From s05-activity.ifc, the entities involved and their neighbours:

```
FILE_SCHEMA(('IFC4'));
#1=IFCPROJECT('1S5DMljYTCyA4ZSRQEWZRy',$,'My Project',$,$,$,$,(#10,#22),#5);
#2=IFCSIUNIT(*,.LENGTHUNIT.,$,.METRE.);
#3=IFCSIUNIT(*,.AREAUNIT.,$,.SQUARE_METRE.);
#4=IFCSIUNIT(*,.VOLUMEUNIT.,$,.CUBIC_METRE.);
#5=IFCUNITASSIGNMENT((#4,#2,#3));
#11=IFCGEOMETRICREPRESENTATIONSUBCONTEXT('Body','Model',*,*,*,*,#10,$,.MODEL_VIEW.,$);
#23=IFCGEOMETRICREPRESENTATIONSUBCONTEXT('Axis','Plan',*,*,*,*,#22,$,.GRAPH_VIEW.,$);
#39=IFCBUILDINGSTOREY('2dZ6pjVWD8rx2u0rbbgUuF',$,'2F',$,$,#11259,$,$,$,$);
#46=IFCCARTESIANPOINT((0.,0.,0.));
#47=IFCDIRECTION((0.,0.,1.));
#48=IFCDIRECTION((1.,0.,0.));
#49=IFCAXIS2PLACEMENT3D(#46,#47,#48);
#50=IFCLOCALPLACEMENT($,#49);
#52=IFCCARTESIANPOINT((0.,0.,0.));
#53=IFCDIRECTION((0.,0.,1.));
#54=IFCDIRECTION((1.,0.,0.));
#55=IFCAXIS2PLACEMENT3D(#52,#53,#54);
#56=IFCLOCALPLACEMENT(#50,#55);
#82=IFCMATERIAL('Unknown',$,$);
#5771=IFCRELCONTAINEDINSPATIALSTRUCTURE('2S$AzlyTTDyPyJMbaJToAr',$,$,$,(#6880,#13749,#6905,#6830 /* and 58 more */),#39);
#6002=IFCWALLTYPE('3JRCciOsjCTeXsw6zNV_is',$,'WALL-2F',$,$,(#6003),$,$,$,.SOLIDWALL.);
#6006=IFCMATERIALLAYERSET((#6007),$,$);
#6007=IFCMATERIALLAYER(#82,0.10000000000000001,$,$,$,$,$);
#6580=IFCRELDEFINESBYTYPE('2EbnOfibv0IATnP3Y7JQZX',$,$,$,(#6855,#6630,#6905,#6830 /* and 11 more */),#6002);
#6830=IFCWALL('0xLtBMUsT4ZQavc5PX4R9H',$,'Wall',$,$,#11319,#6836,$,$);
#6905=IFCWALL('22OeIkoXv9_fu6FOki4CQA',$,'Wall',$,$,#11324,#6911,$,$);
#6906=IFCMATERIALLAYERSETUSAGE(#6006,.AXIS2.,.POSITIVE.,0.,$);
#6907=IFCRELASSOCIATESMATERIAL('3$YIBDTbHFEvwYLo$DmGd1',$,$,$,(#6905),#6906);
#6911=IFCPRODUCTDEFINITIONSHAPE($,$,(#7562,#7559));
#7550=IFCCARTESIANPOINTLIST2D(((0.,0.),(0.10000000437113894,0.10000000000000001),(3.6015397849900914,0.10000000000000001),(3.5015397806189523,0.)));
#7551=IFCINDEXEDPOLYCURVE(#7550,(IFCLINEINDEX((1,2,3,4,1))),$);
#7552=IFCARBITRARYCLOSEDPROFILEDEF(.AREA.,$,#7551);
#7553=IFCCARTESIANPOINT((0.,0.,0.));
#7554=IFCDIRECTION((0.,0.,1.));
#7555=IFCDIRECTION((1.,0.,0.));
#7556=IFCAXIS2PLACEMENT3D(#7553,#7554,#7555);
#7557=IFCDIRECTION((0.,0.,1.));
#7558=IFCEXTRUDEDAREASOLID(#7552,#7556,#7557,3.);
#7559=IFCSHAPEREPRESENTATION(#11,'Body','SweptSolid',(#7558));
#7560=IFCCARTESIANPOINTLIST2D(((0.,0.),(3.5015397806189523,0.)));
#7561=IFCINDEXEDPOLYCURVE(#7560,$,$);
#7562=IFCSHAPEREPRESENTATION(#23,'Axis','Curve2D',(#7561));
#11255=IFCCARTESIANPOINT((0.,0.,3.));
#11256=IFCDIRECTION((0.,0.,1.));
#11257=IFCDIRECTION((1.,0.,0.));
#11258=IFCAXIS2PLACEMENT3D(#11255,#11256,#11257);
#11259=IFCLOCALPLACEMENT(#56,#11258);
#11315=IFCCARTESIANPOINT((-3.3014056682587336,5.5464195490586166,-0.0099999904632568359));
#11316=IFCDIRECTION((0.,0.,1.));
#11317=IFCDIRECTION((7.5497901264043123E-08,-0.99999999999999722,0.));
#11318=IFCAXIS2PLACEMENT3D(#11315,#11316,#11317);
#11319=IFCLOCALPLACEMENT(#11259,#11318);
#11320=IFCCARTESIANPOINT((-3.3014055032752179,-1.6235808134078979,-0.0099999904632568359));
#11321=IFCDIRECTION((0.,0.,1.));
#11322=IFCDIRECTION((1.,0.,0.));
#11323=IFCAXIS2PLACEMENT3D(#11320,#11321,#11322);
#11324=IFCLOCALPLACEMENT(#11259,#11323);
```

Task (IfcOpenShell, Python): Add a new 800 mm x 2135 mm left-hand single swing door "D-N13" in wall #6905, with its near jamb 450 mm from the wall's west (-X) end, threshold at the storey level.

```python
import numpy as np
import ifcopenshell
import ifcopenshell.api.feature
import ifcopenshell.api.geometry
import ifcopenshell.api.root
import ifcopenshell.api.spatial
import ifcopenshell.geom
import ifcopenshell.util.element
import ifcopenshell.util.placement
import ifcopenshell.util.representation
import ifcopenshell.util.shape
import ifcopenshell.util.unit

model = ifcopenshell.open("s05-activity.ifc")
unit_scale = ifcopenshell.util.unit.calculate_unit_scale(model)
settings = ifcopenshell.geom.settings()


def volume(element):
    """Net volume in cubic metres, openings subtracted."""
    shape = ifcopenshell.geom.create_shape(settings, element)
    return ifcopenshell.util.shape.get_volume(shape.geometry)


wall = model.by_guid("22OeIkoXv9_fu6FOki4CQA")
storey = ifcopenshell.util.element.get_container(wall, ifc_class="IfcBuildingStorey")
context = ifcopenshell.util.representation.get_context(model, "Model", "Body", "MODEL_VIEW")
before = volume(wall)

width, height, from_end, sill = 0.8, 2.135, 0.45, 0.0  # metres

# The wall runs along its own X axis, and the end named is its -X end.
wall_shape = ifcopenshell.geom.create_shape(settings, wall)
x, y, z = ifcopenshell.util.shape.get_vertices(wall_shape.geometry).T
start = x.min() + from_end
face, thickness = float(y.min()), float(y.max() - y.min())
wall_matrix = ifcopenshell.util.placement.get_local_placement(wall.ObjectPlacement)
level = ifcopenshell.util.placement.get_local_placement(storey.ObjectPlacement)[2, 3]


def in_wall(x, y):
    """Placement at x, y metres in the wall's axes, at sill height."""
    matrix = wall_matrix.copy()
    matrix[:, 3] = wall_matrix @ np.array([x / unit_scale, y / unit_scale, 0.0, 1.0])
    matrix[2, 3] = level + sill / unit_scale
    return matrix


# Opening: a box that overshoots both wall faces by 50 mm.
opening = ifcopenshell.api.root.create_entity(model, ifc_class="IfcOpeningElement", predefined_type="OPENING")
box = ifcopenshell.api.geometry.add_wall_representation(
    model, context=context, length=width, height=height, thickness=thickness + 0.1
)
ifcopenshell.api.geometry.assign_representation(model, product=opening, representation=box)
ifcopenshell.api.geometry.edit_object_placement(model, product=opening, matrix=in_wall(start, face - 0.05), is_si=False)
ifcopenshell.api.feature.add_feature(model, feature=opening, element=wall)

door = ifcopenshell.api.root.create_entity(model, ifc_class="IfcDoor", name="D-N13", predefined_type="DOOR")
door.OverallWidth, door.OverallHeight = width / unit_scale, height / unit_scale
door.OperationType = "SINGLE_SWING_LEFT"
body = ifcopenshell.api.geometry.add_door_representation(
    model,
    context=context,
    overall_width=door.OverallWidth,
    overall_height=door.OverallHeight,
    operation_type="SINGLE_SWING_LEFT",
    lining_properties={"LiningDepth": thickness / unit_scale, "ThresholdDepth": thickness / unit_scale},
)
ifcopenshell.api.geometry.assign_representation(model, product=door, representation=body)
ifcopenshell.api.spatial.assign_container(model, products=[door], relating_structure=storey)
ifcopenshell.api.feature.add_filling(model, opening=opening, element=door)

# The lining spans the wall, so the door starts at the wall face.
ifcopenshell.api.geometry.edit_object_placement(model, product=door, matrix=in_wall(start, face), is_si=False)

after = volume(wall)

print(f"wall volume {before:.3f} -> {after:.3f} m3")

model.write("s05-activity_v2.ifc")
```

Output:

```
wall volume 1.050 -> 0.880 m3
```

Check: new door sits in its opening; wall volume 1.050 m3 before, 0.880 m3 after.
